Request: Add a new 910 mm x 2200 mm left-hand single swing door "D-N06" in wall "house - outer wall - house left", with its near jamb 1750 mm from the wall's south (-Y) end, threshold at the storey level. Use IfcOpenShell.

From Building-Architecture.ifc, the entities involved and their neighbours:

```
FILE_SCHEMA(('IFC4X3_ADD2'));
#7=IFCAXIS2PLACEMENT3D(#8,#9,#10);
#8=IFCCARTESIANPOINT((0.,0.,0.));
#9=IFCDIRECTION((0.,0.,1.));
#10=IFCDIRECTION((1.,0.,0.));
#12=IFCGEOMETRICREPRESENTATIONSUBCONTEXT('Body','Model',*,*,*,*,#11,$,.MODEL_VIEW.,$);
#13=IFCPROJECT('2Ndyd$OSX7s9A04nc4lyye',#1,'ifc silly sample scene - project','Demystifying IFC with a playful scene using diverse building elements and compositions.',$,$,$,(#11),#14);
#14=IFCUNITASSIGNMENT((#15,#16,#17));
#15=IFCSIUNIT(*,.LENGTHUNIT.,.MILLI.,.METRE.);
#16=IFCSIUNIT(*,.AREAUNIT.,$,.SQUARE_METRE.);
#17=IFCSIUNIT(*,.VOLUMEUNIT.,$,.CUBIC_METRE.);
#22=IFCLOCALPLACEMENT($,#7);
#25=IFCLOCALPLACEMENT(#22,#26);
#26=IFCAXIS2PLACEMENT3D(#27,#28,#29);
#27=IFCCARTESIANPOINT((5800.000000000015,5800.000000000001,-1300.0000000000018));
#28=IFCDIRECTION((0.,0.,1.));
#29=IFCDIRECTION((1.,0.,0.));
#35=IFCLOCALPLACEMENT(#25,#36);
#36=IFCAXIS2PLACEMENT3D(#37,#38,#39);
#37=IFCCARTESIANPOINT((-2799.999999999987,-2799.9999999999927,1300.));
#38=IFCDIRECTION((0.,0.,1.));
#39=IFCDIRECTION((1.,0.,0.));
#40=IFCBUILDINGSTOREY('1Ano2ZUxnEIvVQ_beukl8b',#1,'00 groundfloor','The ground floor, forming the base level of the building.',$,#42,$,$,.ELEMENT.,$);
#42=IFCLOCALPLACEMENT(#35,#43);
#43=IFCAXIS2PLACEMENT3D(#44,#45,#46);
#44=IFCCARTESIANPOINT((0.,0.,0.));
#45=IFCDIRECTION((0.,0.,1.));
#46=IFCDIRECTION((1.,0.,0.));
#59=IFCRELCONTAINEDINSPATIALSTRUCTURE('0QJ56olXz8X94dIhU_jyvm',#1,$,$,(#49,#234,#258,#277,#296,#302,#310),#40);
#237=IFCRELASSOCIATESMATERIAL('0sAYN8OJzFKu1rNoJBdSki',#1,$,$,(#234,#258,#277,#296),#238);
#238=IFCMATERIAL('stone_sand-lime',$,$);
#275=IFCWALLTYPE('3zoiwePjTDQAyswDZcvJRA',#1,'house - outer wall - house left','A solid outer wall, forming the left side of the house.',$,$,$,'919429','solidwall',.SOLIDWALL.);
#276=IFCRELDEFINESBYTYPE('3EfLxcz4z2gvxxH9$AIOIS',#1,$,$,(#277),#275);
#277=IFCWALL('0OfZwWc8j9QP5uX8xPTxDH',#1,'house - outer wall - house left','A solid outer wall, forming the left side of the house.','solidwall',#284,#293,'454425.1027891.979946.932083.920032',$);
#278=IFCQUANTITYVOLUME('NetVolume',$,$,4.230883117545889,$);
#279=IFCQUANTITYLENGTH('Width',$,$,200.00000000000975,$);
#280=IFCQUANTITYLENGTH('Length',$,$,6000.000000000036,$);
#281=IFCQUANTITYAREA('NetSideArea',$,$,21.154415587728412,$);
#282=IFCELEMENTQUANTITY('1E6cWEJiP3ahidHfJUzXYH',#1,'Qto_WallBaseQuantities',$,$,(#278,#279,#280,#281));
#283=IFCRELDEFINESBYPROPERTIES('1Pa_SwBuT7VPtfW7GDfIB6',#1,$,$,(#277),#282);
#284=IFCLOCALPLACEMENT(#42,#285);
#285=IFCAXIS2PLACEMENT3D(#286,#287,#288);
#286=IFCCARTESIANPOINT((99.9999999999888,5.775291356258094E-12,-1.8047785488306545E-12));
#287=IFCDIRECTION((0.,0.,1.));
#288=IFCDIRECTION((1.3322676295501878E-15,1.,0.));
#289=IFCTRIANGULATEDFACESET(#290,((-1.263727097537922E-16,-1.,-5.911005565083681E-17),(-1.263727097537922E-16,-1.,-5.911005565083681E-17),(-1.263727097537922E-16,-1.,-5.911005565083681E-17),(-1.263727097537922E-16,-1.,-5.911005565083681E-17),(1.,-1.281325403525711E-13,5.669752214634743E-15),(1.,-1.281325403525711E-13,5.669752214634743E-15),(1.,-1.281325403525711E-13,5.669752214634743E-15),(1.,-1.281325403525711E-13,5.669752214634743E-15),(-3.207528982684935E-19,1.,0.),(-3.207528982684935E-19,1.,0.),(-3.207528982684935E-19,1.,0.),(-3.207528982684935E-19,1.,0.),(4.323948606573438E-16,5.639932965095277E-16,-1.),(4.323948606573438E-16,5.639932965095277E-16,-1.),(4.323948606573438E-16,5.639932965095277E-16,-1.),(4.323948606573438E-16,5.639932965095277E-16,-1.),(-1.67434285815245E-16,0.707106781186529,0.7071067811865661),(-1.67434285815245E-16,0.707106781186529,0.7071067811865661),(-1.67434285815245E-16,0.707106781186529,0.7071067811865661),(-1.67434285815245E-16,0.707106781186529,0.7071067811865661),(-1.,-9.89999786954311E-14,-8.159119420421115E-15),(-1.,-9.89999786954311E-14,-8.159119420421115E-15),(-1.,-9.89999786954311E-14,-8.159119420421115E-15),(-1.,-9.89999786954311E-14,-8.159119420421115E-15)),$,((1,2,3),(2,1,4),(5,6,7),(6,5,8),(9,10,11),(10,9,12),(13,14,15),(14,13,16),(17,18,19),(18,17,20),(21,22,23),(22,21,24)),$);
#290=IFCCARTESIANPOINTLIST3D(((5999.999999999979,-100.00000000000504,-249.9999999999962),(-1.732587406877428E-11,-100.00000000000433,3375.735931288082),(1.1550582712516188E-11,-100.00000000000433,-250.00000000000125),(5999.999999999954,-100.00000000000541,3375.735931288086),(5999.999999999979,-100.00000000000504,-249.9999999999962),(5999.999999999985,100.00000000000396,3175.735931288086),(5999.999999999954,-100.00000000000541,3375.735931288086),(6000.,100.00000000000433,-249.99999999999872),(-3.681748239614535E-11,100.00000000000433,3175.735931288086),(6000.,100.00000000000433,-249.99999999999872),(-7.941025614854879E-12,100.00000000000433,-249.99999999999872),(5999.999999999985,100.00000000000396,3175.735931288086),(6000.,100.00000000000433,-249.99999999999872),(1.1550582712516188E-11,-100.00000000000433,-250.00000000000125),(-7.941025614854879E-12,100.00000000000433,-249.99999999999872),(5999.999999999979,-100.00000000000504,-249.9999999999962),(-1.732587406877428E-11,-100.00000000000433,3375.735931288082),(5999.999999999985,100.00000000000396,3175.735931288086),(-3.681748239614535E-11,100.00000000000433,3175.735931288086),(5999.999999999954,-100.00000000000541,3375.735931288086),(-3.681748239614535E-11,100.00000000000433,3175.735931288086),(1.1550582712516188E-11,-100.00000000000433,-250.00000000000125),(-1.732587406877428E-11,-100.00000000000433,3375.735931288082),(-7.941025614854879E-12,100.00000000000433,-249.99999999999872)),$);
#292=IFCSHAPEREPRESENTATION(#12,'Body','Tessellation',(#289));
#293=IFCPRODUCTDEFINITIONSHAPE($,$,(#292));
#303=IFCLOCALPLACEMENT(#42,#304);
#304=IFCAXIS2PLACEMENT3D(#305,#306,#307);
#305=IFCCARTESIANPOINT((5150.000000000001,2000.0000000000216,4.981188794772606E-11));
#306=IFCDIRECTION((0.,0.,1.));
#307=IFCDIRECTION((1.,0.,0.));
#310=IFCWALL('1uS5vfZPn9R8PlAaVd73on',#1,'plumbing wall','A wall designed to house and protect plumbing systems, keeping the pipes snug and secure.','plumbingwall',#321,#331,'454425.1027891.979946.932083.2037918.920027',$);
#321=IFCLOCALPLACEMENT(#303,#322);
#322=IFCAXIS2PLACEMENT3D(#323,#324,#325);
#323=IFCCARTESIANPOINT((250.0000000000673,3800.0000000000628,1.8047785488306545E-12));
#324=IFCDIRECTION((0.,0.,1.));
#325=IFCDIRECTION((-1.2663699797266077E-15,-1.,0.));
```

```python
import numpy as np
import ifcopenshell
import ifcopenshell.api.feature
import ifcopenshell.api.geometry
import ifcopenshell.api.pset
import ifcopenshell.api.root
import ifcopenshell.api.spatial
import ifcopenshell.geom
import ifcopenshell.util.element
import ifcopenshell.util.placement
import ifcopenshell.util.representation
import ifcopenshell.util.shape
import ifcopenshell.util.unit

model = ifcopenshell.open("Building-Architecture.ifc")
unit_scale = ifcopenshell.util.unit.calculate_unit_scale(model)
area_scale = ifcopenshell.util.unit.calculate_unit_scale(model, "AREAUNIT")
volume_scale = ifcopenshell.util.unit.calculate_unit_scale(model, "VOLUMEUNIT")
settings = ifcopenshell.geom.settings()


def volume(element):
    """Net volume in cubic metres, openings subtracted."""
    shape = ifcopenshell.geom.create_shape(settings, element)
    return ifcopenshell.util.shape.get_volume(shape.geometry)


wall = model.by_guid("0OfZwWc8j9QP5uX8xPTxDH")
storey = ifcopenshell.util.element.get_container(wall, ifc_class="IfcBuildingStorey")
context = ifcopenshell.util.representation.get_context(model, "Model", "Body", "MODEL_VIEW")
before = volume(wall)

width, height, from_end, sill = 0.91, 2.2, 1.75, 0.0  # metres

# The wall runs along its own X axis, and the end named is its -X end.
wall_shape = ifcopenshell.geom.create_shape(settings, wall)
x, y, z = ifcopenshell.util.shape.get_vertices(wall_shape.geometry).T
start = x.min() + from_end
face, thickness = float(y.min()), float(y.max() - y.min())
wall_matrix = ifcopenshell.util.placement.get_local_placement(wall.ObjectPlacement)
level = ifcopenshell.util.placement.get_local_placement(storey.ObjectPlacement)[2, 3]


def in_wall(x, y):
    """Placement at x, y metres in the wall's axes, at sill height."""
    matrix = wall_matrix.copy()
    matrix[:, 3] = wall_matrix @ np.array([x / unit_scale, y / unit_scale, 0.0, 1.0])
    matrix[2, 3] = level + sill / unit_scale
    return matrix


# Opening: a box that overshoots both wall faces by 50 mm.
opening = ifcopenshell.api.root.create_entity(model, ifc_class="IfcOpeningElement", predefined_type="OPENING")
box = ifcopenshell.api.geometry.add_wall_representation(
    model, context=context, length=width, height=height, thickness=thickness + 0.1
)
ifcopenshell.api.geometry.assign_representation(model, product=opening, representation=box)
ifcopenshell.api.geometry.edit_object_placement(model, product=opening, matrix=in_wall(start, face - 0.05), is_si=False)
ifcopenshell.api.feature.add_feature(model, feature=opening, element=wall)

door = ifcopenshell.api.root.create_entity(model, ifc_class="IfcDoor", name="D-N06", predefined_type="DOOR")
door.OverallWidth, door.OverallHeight = width / unit_scale, height / unit_scale
door.OperationType = "SINGLE_SWING_LEFT"
body = ifcopenshell.api.geometry.add_door_representation(
    model,
    context=context,
    overall_width=door.OverallWidth,
    overall_height=door.OverallHeight,
    operation_type="SINGLE_SWING_LEFT",
    lining_properties={"LiningDepth": thickness / unit_scale, "ThresholdDepth": thickness / unit_scale},
)
ifcopenshell.api.geometry.assign_representation(model, product=door, representation=body)
ifcopenshell.api.spatial.assign_container(model, products=[door], relating_structure=storey)
ifcopenshell.api.feature.add_filling(model, opening=opening, element=door)

# The lining spans the wall, so the door starts at the wall face.
ifcopenshell.api.geometry.edit_object_placement(model, product=door, matrix=in_wall(start, face), is_si=False)

after = volume(wall)

# Update the wall's stored quantities.
qto = model.by_id(ifcopenshell.util.element.get_pset(wall, "Qto_WallBaseQuantities", should_inherit=False)["id"])
ifcopenshell.api.pset.edit_qto(model, qto=qto, properties={
    "NetVolume": after / volume_scale,
    "NetSideArea": after / thickness / area_scale,
})

print(f"wall volume {before:.3f} -> {after:.3f} m3")

model.write("Building-Architecture-out.ifc")
```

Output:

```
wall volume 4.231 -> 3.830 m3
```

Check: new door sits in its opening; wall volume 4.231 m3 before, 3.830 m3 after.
